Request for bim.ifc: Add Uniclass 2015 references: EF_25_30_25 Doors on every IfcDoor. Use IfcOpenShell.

First a look at what the model holds.

```python
import ifcopenshell

model = ifcopenshell.open("bim.ifc")
print(model.schema)
print("classifications:", [c.Name for c in model.by_type("IfcClassification")])
for ifc_class in ("IfcDoor", "IfcRoof", "IfcStair", "IfcWall", "IfcWindow"):
    print(ifc_class, len(model.by_type(ifc_class)))
```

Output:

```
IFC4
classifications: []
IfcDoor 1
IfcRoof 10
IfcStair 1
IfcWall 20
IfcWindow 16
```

```python
import ifcopenshell
import ifcopenshell.api.classification

model = ifcopenshell.open("bim.ifc")

system = ifcopenshell.api.classification.add_classification(model, classification="Uniclass 2015")

codes = {
    "IfcDoor": ("EF_25_30_25", "Doors"),
}
for ifc_class, (code, name) in codes.items():
    products = model.by_type(ifc_class)
    ifcopenshell.api.classification.add_reference(
        model, products=products, classification=system, identification=code, name=name
    )
    print(code, len(products))

model.write("bim_v2.ifc")
```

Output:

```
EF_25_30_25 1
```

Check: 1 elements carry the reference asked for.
